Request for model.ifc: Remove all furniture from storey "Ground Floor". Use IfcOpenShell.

First a look at what the model holds.

```python
import ifcopenshell
import ifcopenshell.util.element

model = ifcopenshell.open("model.ifc")
print(model.schema)
storey = next(s for s in model.by_type("IfcBuildingStorey") if s.Name == "Ground Floor")
furniture = [e for e in ifcopenshell.util.element.get_decomposition(storey) if e.is_a("IfcFurnishingElement")]
seen = {}
for e in furniture:
    element_type = ifcopenshell.util.element.get_type(e)
    name = element_type.Name if element_type not in (None, e) else None
    seen[name] = seen.get(name, 0) + 1
for name, count in sorted(seen.items(), key=str):
    print(count, "x", name)
```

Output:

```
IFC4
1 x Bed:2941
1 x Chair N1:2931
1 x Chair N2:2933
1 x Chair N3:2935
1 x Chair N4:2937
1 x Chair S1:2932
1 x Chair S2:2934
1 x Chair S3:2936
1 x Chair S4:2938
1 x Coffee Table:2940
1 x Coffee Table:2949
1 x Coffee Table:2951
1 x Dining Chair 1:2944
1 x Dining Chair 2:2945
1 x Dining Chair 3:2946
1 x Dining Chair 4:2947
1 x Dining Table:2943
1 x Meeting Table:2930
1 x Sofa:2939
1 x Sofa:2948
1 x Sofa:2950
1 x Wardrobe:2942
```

```python
import ifcopenshell
import ifcopenshell.api.root
import ifcopenshell.util.element

model = ifcopenshell.open("model.ifc")

storey = next(s for s in model.by_type("IfcBuildingStorey") if s.Name == "Ground Floor")
furniture = [e for e in ifcopenshell.util.element.get_decomposition(storey) if e.is_a("IfcFurnishingElement")]

for e in furniture:
    ifcopenshell.api.root.remove_product(model, product=e)
print(len(furniture), "removed")

model.write("model_v2.ifc")
```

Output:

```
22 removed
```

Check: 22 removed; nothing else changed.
